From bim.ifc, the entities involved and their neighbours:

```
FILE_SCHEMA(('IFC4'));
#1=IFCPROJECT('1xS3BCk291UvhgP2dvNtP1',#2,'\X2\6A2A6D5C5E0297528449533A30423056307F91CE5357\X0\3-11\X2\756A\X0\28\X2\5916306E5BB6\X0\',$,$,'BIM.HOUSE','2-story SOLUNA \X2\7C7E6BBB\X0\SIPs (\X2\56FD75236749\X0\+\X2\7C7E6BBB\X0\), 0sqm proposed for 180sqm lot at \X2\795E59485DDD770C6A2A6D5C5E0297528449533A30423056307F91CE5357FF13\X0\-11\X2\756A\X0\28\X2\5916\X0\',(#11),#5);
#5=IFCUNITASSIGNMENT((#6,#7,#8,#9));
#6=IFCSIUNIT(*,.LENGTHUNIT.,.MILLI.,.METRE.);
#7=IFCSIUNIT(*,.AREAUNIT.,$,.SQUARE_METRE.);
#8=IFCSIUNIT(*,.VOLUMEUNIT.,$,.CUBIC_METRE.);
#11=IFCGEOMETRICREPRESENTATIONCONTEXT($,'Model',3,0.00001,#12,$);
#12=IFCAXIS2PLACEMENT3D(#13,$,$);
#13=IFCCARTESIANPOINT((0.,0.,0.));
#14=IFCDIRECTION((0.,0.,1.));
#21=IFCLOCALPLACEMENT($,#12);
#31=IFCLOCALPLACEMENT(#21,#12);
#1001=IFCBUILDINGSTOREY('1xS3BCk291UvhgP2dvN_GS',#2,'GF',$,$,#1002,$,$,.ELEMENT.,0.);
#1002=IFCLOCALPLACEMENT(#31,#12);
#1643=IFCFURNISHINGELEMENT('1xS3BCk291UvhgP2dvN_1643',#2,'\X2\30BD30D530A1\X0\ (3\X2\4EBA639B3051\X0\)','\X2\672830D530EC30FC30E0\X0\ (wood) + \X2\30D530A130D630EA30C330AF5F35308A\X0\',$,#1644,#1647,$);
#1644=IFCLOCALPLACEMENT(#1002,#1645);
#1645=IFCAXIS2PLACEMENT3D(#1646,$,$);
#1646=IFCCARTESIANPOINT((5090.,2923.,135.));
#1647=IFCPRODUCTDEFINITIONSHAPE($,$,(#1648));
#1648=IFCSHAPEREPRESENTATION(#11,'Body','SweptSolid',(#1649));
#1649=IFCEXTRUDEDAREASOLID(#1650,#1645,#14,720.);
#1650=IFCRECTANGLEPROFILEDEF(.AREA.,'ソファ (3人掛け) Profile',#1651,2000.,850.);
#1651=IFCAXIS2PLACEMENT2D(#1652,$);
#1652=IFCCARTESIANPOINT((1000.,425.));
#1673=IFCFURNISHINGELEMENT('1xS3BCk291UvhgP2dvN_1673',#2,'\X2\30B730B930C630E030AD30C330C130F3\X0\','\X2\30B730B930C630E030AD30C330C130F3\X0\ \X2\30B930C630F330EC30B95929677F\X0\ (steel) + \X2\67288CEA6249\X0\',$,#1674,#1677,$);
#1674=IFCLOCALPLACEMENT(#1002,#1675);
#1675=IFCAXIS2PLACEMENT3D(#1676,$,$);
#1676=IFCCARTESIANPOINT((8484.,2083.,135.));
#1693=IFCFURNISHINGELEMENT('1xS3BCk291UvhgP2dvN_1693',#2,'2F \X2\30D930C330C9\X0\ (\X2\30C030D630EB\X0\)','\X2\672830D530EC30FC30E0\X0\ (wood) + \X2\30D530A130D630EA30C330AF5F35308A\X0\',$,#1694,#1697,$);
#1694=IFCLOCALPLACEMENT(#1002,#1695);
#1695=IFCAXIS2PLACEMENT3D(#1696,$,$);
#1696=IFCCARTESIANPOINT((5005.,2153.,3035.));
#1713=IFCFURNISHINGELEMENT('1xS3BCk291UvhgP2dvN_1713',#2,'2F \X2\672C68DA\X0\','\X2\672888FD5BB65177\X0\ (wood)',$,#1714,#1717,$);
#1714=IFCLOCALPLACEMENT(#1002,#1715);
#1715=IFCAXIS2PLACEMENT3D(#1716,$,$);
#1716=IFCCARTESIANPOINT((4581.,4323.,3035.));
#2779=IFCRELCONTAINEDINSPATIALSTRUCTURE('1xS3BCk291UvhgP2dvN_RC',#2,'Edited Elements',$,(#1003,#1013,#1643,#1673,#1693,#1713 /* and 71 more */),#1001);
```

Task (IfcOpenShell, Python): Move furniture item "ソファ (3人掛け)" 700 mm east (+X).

```python
import ifcopenshell
import ifcopenshell.api.geometry
import ifcopenshell.util.placement
import ifcopenshell.util.unit

model = ifcopenshell.open("bim.ifc")
unit_scale = ifcopenshell.util.unit.calculate_unit_scale(model)

item = model.by_id(1643)
matrix = ifcopenshell.util.placement.get_local_placement(item.ObjectPlacement)
matrix[0, 3] += 0.7 / unit_scale
ifcopenshell.api.geometry.edit_object_placement(model, product=item, matrix=matrix, is_si=False)

print(ifcopenshell.util.placement.get_local_placement(item.ObjectPlacement).round(3) + 0.0)

model.write("bim_v2.ifc")
```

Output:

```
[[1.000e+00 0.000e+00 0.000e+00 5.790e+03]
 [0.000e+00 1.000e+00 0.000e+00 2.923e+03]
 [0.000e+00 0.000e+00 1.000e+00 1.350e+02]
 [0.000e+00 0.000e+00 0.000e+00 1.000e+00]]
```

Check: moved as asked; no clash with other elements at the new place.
